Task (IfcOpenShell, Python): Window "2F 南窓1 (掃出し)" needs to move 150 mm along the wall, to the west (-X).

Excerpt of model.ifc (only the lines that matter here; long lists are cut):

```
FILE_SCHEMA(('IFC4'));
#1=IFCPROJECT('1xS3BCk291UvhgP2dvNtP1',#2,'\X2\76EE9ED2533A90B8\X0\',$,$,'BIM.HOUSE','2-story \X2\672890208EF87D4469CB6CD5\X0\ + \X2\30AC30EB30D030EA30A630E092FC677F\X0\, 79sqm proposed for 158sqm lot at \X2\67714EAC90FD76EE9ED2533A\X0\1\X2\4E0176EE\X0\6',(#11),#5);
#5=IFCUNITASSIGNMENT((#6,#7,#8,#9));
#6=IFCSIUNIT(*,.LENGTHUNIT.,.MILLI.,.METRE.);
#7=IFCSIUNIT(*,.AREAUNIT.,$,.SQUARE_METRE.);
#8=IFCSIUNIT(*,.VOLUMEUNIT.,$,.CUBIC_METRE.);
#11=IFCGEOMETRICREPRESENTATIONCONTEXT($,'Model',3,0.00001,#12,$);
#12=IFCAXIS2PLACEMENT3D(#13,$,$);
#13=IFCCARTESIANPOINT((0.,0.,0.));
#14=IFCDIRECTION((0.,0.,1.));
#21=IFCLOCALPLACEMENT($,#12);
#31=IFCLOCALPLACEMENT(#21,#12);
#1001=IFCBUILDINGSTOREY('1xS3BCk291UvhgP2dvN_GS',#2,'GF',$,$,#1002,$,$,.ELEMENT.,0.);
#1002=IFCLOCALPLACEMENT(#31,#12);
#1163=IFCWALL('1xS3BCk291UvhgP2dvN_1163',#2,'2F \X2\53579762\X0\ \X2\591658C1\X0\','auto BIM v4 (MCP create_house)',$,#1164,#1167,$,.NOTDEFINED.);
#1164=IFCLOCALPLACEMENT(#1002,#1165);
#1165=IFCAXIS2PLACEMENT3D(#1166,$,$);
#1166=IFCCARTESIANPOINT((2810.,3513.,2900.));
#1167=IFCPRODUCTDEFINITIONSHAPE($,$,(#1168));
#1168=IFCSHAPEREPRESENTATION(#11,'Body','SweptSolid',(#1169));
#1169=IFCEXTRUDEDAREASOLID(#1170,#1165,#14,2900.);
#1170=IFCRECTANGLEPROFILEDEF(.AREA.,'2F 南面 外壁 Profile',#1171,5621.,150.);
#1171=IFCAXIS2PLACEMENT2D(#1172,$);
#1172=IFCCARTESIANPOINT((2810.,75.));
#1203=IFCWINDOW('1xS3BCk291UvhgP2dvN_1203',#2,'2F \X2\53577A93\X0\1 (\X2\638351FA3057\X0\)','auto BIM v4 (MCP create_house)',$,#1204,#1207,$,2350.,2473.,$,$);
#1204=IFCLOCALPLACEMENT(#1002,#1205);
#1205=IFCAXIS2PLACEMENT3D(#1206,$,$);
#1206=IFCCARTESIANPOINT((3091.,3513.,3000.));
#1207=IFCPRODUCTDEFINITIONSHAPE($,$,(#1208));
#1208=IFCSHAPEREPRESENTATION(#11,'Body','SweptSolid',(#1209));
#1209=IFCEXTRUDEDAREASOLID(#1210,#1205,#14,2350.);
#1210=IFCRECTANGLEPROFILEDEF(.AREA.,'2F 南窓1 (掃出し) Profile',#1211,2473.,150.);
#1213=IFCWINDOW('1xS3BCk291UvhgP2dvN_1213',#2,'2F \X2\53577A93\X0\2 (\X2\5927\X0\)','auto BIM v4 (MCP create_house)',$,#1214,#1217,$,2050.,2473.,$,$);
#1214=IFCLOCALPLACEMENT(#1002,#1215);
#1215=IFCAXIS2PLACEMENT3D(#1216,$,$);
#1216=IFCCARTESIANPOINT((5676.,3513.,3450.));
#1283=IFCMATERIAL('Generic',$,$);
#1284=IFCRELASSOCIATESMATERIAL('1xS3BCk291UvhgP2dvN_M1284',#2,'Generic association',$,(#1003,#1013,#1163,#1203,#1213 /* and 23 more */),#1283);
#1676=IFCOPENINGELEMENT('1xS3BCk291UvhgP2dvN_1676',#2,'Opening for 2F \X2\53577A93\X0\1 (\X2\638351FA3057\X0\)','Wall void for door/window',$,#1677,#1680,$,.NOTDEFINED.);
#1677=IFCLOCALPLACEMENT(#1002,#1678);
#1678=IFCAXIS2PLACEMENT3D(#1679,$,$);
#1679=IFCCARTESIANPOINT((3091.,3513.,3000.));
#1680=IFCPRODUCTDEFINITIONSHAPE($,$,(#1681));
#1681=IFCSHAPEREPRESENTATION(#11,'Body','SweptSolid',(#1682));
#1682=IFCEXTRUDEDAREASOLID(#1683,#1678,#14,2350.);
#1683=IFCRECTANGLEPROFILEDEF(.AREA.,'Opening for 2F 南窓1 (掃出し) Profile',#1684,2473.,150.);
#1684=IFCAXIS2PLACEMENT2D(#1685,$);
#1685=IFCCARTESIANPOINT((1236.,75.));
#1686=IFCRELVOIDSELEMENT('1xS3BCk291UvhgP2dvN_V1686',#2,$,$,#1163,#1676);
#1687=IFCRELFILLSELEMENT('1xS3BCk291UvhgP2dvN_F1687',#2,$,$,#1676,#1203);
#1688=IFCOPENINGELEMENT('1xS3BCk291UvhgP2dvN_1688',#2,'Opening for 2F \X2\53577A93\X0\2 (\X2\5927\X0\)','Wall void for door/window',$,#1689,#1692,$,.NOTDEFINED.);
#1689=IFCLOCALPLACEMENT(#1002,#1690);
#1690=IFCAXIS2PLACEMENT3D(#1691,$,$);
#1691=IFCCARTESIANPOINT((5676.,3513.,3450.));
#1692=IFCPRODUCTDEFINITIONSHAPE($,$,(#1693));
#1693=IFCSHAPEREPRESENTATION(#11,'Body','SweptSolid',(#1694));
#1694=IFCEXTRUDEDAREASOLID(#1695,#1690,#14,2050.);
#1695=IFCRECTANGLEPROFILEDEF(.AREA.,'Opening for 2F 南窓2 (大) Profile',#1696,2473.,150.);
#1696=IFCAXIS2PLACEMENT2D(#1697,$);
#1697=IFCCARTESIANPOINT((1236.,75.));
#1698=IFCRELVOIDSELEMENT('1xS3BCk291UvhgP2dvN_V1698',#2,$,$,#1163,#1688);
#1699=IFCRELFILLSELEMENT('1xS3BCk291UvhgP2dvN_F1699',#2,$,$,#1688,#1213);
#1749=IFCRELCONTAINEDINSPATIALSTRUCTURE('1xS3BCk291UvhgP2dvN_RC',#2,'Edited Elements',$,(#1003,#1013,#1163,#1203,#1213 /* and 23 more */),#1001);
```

```python
import ifcopenshell
import ifcopenshell.api.geometry
import ifcopenshell.util.placement
import ifcopenshell.util.unit

model = ifcopenshell.open("model.ifc")
unit_scale = ifcopenshell.util.unit.calculate_unit_scale(model)

window = model.by_id(1203)
opening = window.FillsVoids[0].RelatingOpeningElement
wall = opening.VoidsElements[0].RelatingBuildingElement

wall_matrix = ifcopenshell.util.placement.get_local_placement(wall.ObjectPlacement)
shift = wall_matrix[:3, 0] * -0.15 / unit_scale
before = ifcopenshell.util.placement.get_local_placement(window.ObjectPlacement)[:3, 3].copy()

# The window is not placed relative to its opening, so move both.
for product in (opening, window):
    matrix = ifcopenshell.util.placement.get_local_placement(product.ObjectPlacement)
    matrix[:3, 3] += shift
    ifcopenshell.api.geometry.edit_object_placement(model, product=product, matrix=matrix, is_si=False)

after = ifcopenshell.util.placement.get_local_placement(window.ObjectPlacement)[:3, 3]
print("window moved by", (after - before).round(3) + 0.0)

model.write("model_rev.ifc")
```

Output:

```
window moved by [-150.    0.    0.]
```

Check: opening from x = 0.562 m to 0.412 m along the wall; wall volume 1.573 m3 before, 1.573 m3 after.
